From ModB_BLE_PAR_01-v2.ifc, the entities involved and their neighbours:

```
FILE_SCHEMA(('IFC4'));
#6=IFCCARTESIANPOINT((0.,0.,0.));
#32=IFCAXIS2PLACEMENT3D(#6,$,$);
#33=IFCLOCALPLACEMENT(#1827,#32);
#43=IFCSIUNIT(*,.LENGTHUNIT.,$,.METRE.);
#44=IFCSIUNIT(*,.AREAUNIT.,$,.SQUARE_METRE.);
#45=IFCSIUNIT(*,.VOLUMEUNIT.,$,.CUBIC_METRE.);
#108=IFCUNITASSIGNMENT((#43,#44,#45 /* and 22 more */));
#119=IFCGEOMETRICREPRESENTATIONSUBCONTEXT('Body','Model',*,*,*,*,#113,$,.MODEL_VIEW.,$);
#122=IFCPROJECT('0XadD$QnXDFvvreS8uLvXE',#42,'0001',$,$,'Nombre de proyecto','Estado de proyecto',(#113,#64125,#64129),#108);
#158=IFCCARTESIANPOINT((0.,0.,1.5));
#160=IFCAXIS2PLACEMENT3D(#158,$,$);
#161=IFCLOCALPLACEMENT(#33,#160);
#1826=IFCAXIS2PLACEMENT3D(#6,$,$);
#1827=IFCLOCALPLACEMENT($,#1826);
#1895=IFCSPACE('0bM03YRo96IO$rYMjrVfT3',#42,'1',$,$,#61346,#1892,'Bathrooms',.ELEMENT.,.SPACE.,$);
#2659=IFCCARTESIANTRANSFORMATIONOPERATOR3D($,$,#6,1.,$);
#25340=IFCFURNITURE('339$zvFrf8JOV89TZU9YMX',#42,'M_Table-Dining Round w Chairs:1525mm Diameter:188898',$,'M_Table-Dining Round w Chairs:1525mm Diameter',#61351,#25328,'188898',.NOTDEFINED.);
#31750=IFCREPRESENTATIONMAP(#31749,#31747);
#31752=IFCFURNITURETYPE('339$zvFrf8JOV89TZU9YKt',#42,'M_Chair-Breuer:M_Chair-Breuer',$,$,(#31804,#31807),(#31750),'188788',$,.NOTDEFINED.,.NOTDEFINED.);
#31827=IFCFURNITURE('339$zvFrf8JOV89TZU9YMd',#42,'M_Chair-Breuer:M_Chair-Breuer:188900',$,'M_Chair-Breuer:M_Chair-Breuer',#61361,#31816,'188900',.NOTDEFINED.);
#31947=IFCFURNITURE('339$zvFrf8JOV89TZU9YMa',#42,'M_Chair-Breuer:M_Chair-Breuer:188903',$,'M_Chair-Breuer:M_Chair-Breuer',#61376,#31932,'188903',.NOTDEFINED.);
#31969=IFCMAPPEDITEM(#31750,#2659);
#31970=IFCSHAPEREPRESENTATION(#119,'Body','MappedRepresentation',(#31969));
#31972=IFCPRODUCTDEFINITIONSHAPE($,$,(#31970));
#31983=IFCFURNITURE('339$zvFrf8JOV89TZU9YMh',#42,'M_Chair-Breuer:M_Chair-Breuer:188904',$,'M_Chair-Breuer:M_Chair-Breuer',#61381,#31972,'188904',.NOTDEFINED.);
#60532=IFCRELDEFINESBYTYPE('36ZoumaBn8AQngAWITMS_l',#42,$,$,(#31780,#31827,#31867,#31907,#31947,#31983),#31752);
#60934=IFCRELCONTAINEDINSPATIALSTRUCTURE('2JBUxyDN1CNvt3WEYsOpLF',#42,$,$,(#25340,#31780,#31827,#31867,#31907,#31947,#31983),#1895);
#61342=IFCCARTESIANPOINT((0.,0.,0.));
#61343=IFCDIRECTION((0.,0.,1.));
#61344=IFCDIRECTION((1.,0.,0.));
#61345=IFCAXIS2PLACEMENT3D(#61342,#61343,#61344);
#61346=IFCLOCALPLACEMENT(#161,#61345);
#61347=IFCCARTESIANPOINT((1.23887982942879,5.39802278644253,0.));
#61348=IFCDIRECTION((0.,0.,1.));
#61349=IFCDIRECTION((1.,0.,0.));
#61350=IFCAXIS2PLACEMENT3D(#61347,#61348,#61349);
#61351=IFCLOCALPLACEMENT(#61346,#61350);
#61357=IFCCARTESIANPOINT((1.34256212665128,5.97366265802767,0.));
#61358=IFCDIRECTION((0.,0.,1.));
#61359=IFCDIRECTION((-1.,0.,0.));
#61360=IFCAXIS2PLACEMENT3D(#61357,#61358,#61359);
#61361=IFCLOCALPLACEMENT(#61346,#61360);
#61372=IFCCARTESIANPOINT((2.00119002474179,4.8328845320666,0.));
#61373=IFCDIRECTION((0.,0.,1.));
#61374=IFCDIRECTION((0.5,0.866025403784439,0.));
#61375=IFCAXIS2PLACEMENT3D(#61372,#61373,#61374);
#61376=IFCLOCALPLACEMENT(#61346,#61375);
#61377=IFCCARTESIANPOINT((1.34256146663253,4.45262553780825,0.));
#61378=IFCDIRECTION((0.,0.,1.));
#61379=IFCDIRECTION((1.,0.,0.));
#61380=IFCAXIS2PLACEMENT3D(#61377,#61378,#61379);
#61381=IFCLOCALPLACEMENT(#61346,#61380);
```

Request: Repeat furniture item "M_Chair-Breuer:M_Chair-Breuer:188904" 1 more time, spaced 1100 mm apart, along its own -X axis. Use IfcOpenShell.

```python
import ifcopenshell
import ifcopenshell.api.geometry
import ifcopenshell.api.root
import ifcopenshell.util.element
import ifcopenshell.util.placement

model = ifcopenshell.open("ModB_BLE_PAR_01-v2.ifc")


def reuse_history(source, copy):
    """copy_class also copies each property set's owner history, people and application; keep the originals."""
    for rel in copy.IsDefinedBy:
        if rel.is_a("IfcRelDefinesByProperties") and (history := rel.RelatingPropertyDefinition.OwnerHistory):
            rel.RelatingPropertyDefinition.OwnerHistory = source.OwnerHistory
            ifcopenshell.util.element.remove_deep2(model, history)


source = model.by_guid("339$zvFrf8JOV89TZU9YMh")
base = ifcopenshell.util.placement.get_local_placement(source.ObjectPlacement)
step = -base[:3, 0] * 1.1

for i in range(1, 2):
    copy = ifcopenshell.api.root.copy_class(model, product=source)
    copy.Representation = ifcopenshell.util.element.copy_deep(
        model, source.Representation, exclude=["IfcGeometricRepresentationContext", "IfcRepresentationMap"]
    )
    copy.Name = "M_Chair-Breuer:M_Chair-Breuer"
    copy.Tag = None
    reuse_history(source, copy)
    matrix = base.copy()
    matrix[:3, 3] += i * step
    print("added at", matrix[:3, 3].round(3) + 0.0)
    ifcopenshell.api.geometry.edit_object_placement(model, product=copy, matrix=matrix, is_si=False)

model.write("ModB_BLE_PAR_01-v2-out.ifc")
```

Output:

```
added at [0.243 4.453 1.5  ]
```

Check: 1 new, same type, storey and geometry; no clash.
